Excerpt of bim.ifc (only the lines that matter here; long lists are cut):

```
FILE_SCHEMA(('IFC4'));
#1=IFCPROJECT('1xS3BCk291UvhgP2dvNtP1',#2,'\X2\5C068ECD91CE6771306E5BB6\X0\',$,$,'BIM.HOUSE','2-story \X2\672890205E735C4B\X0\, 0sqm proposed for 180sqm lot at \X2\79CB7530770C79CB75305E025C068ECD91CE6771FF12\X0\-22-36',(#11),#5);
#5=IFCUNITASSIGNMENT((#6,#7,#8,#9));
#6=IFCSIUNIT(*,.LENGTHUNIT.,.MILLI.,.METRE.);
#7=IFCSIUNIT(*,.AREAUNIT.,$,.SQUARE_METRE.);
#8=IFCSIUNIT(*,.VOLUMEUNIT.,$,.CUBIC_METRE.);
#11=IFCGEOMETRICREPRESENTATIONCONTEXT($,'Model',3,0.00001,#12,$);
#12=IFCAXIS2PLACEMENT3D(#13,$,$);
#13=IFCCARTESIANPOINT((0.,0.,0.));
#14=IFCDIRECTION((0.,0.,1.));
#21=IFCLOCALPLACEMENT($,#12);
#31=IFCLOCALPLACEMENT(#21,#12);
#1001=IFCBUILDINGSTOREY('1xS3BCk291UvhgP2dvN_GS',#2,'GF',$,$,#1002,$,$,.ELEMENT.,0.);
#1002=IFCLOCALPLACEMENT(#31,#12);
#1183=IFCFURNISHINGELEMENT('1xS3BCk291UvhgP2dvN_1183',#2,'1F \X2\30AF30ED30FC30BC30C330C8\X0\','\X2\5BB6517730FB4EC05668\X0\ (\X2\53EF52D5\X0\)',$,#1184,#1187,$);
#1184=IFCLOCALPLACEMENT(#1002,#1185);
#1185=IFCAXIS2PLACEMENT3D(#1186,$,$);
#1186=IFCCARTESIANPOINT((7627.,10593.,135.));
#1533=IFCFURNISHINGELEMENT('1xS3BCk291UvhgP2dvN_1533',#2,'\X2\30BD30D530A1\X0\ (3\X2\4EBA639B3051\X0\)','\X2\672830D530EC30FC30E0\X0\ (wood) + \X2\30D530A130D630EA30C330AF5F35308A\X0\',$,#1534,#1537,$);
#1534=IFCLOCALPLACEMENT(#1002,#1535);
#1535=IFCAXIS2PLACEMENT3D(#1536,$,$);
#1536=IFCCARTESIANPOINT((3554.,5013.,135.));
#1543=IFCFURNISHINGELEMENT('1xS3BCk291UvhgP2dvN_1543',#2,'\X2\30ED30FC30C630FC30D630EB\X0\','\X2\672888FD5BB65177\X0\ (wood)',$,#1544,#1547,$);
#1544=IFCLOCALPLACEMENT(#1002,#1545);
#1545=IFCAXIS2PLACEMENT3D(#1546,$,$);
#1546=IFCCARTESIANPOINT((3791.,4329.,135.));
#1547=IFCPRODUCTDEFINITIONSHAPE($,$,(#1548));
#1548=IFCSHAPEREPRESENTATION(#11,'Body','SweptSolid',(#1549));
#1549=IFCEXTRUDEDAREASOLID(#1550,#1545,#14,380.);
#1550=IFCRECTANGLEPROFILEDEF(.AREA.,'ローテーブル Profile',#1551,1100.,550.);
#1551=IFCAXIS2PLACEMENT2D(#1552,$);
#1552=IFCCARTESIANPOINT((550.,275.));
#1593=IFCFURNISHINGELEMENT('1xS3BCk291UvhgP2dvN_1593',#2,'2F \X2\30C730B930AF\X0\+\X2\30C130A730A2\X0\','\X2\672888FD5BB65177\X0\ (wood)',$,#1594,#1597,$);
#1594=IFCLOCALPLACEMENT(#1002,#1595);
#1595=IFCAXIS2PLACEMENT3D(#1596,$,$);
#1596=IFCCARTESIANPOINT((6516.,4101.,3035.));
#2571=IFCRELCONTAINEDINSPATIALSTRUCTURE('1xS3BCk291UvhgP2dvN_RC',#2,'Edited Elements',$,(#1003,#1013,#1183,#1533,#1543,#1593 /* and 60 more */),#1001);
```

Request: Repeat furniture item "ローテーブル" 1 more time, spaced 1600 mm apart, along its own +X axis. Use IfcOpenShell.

```python
import ifcopenshell
import ifcopenshell.api.geometry
import ifcopenshell.api.root
import ifcopenshell.util.element
import ifcopenshell.util.placement

model = ifcopenshell.open("bim.ifc")


def reuse_history(source, copy):
    """copy_class also copies each property set's owner history, people and application; keep the originals."""
    for rel in copy.IsDefinedBy:
        if rel.is_a("IfcRelDefinesByProperties") and (history := rel.RelatingPropertyDefinition.OwnerHistory):
            rel.RelatingPropertyDefinition.OwnerHistory = source.OwnerHistory
            ifcopenshell.util.element.remove_deep2(model, history)


source = model.by_guid("1xS3BCk291UvhgP2dvN_1543")
base = ifcopenshell.util.placement.get_local_placement(source.ObjectPlacement)
step = base[:3, 0] * 1600.0

for i in range(1, 2):
    copy = ifcopenshell.api.root.copy_class(model, product=source)
    copy.Representation = ifcopenshell.util.element.copy_deep(
        model, source.Representation, exclude=["IfcGeometricRepresentationContext", "IfcRepresentationMap"]
    )
    reuse_history(source, copy)
    matrix = base.copy()
    matrix[:3, 3] += i * step
    print("added at", matrix[:3, 3].round(3) + 0.0)
    ifcopenshell.api.geometry.edit_object_placement(model, product=copy, matrix=matrix, is_si=False)

model.write("bim-out.ifc")
```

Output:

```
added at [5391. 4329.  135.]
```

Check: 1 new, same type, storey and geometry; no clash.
